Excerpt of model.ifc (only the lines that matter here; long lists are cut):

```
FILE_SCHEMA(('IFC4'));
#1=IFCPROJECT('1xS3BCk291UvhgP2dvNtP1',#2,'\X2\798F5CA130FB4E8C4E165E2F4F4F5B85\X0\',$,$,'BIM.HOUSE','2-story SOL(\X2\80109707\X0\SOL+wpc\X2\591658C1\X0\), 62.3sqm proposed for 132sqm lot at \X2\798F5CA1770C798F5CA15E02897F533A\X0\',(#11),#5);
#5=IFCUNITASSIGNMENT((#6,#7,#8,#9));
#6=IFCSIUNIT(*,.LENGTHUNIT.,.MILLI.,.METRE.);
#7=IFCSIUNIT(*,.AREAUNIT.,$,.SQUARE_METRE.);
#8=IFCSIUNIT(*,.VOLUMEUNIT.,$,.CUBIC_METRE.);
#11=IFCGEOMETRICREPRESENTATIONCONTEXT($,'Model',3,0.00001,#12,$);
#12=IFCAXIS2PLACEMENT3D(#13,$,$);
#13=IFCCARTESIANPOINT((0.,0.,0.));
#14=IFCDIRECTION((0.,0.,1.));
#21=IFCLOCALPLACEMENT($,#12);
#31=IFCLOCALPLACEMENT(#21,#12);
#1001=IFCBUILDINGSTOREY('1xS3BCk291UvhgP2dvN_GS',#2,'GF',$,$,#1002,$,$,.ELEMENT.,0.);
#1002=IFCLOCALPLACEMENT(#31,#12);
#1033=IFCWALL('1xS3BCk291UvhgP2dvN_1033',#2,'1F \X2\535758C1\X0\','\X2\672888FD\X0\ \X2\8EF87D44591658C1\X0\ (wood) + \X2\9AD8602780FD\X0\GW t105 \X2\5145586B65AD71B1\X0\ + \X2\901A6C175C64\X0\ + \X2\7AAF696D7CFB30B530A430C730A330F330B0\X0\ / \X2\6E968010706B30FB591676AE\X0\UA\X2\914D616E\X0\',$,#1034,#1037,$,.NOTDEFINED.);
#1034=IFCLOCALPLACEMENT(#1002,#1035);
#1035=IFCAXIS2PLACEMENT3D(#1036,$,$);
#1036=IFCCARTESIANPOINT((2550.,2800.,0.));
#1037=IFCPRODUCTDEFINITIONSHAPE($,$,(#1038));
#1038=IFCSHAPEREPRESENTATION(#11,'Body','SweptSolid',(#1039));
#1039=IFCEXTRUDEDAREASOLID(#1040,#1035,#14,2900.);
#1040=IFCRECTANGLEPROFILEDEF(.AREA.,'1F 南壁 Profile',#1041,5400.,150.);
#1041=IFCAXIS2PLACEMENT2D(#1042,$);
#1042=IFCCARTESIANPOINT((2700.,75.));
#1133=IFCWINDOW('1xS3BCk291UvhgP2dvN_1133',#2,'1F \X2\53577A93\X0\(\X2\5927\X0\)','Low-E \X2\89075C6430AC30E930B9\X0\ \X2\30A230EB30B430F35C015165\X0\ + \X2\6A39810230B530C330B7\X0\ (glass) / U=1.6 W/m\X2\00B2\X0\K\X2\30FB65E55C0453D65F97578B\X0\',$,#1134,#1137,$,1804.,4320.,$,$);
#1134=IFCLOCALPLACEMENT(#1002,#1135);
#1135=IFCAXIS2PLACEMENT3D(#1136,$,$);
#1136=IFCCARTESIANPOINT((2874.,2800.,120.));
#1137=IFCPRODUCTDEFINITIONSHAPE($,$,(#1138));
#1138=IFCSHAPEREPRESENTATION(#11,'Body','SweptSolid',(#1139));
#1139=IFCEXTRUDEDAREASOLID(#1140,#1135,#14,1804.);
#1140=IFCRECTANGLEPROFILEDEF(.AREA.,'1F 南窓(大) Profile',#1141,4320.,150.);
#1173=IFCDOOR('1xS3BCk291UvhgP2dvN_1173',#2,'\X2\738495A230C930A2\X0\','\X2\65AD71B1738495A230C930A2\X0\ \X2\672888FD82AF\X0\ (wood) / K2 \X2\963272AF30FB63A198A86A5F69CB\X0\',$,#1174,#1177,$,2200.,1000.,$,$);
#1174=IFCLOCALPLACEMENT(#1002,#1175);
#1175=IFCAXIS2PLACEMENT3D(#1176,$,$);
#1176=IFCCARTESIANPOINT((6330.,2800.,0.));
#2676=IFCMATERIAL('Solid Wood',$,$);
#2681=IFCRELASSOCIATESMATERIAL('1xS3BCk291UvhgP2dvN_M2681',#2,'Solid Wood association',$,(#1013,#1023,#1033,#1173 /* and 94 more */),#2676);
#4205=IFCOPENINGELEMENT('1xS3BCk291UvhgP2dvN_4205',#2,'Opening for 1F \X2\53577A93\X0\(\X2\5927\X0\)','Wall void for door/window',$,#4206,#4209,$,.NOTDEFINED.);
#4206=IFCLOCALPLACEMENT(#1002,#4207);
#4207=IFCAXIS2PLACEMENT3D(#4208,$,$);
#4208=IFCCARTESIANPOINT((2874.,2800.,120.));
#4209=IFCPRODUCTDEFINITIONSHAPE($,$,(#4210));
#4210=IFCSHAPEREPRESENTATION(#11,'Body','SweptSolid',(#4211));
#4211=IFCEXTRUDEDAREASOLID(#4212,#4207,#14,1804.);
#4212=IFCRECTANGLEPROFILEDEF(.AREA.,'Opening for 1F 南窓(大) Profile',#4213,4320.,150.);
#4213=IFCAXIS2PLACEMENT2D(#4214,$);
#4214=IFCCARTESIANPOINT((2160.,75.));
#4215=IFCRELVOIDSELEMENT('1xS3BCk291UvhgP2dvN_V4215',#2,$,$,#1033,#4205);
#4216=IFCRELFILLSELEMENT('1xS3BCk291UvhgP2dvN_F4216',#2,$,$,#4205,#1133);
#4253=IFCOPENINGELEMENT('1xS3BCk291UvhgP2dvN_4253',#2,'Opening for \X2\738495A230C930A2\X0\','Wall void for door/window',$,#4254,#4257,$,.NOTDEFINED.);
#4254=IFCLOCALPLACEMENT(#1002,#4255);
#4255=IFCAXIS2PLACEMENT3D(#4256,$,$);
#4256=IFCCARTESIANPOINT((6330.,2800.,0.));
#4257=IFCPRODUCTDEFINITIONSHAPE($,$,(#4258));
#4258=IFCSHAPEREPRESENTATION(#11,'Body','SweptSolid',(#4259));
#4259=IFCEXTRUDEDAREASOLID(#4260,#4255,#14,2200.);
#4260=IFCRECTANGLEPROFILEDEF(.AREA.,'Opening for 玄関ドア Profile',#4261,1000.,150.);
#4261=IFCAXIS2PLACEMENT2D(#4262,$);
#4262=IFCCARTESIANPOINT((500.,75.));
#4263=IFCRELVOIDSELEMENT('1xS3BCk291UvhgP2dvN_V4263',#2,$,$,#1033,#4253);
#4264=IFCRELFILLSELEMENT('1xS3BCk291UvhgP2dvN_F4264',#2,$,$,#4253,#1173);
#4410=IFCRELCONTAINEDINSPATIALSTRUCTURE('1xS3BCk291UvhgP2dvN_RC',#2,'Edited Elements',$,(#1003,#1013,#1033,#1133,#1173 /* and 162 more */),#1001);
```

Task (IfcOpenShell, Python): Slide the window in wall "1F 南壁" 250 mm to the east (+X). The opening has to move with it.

```python
import ifcopenshell
import ifcopenshell.api.geometry
import ifcopenshell.util.placement

model = ifcopenshell.open("model.ifc")

window = model.by_guid("1xS3BCk291UvhgP2dvN_1133")
opening = window.FillsVoids[0].RelatingOpeningElement
wall = opening.VoidsElements[0].RelatingBuildingElement

wall_matrix = ifcopenshell.util.placement.get_local_placement(wall.ObjectPlacement)
shift = wall_matrix[:3, 0] * 250.0
before = ifcopenshell.util.placement.get_local_placement(window.ObjectPlacement)[:3, 3].copy()

# The window is not placed relative to its opening, so move both.
for product in (opening, window):
    matrix = ifcopenshell.util.placement.get_local_placement(product.ObjectPlacement)
    matrix[:3, 3] += shift
    ifcopenshell.api.geometry.edit_object_placement(model, product=product, matrix=matrix, is_si=False)

after = ifcopenshell.util.placement.get_local_placement(window.ObjectPlacement)[:3, 3]
print("window moved by", (after - before).round(3) + 0.0)

model.write("model_v2.ifc")
```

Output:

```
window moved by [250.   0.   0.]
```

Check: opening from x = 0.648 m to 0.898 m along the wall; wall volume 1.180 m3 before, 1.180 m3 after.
